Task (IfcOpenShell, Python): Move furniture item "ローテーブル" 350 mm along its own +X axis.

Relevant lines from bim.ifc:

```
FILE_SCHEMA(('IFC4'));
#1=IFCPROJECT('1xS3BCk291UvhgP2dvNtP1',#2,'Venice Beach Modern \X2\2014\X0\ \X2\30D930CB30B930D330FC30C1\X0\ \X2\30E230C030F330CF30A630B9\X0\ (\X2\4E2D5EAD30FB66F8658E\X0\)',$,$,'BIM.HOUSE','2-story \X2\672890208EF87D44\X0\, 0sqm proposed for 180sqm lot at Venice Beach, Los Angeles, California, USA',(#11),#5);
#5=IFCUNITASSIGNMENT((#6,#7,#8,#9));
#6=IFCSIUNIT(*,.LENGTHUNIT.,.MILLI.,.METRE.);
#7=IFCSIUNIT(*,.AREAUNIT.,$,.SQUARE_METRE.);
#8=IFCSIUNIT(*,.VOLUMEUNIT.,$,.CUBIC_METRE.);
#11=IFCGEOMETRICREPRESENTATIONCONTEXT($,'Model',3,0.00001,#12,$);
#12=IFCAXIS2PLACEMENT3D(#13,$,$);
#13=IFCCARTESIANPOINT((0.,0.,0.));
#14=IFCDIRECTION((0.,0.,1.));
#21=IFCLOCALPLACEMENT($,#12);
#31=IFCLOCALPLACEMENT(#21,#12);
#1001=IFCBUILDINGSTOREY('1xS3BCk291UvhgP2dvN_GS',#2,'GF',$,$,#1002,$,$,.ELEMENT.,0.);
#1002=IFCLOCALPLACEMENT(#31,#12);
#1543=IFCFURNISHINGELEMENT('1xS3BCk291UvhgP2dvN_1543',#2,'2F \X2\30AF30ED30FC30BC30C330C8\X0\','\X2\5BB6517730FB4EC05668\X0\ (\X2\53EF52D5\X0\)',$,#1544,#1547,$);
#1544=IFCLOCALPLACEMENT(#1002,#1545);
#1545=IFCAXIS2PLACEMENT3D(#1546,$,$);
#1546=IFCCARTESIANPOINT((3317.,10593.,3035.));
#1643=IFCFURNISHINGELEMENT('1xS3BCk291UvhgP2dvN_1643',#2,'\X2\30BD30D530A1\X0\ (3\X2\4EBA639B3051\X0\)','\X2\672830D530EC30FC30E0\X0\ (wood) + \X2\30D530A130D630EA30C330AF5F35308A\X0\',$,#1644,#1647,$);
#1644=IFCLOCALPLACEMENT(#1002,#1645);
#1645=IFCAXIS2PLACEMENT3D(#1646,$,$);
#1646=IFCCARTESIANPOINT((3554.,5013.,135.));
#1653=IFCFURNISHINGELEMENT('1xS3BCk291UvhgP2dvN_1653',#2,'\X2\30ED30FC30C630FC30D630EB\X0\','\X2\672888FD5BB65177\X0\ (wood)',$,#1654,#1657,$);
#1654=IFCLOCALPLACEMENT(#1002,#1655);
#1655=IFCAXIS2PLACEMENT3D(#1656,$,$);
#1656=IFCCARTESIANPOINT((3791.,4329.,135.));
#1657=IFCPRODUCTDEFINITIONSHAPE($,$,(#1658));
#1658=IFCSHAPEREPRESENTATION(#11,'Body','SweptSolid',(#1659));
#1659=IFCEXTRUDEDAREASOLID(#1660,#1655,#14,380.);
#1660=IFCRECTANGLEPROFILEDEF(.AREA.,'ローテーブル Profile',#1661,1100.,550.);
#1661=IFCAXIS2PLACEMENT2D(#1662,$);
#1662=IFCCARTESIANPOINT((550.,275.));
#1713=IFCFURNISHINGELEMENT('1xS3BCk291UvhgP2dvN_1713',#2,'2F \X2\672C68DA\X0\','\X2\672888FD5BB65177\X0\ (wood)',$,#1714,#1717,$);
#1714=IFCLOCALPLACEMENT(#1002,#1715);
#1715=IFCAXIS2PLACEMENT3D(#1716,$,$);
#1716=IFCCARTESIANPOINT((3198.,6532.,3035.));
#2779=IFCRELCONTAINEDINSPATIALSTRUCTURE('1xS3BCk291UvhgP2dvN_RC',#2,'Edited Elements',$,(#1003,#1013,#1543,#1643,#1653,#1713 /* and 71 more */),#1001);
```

```python
import ifcopenshell
import ifcopenshell.api.geometry
import ifcopenshell.util.placement
import ifcopenshell.util.unit

model = ifcopenshell.open("bim.ifc")
unit_scale = ifcopenshell.util.unit.calculate_unit_scale(model)

item = model.by_guid("1xS3BCk291UvhgP2dvN_1653")
matrix = ifcopenshell.util.placement.get_local_placement(item.ObjectPlacement)
matrix[:3, 3] += matrix[:3, 0] * 0.35 / unit_scale
ifcopenshell.api.geometry.edit_object_placement(model, product=item, matrix=matrix, is_si=False)

print(ifcopenshell.util.placement.get_local_placement(item.ObjectPlacement).round(3) + 0.0)

model.write("bim_rev.ifc")
```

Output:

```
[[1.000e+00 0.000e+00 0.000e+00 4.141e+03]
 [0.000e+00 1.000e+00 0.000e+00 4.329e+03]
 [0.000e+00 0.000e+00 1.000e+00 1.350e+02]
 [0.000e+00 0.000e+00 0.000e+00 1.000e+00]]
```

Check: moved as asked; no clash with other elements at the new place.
